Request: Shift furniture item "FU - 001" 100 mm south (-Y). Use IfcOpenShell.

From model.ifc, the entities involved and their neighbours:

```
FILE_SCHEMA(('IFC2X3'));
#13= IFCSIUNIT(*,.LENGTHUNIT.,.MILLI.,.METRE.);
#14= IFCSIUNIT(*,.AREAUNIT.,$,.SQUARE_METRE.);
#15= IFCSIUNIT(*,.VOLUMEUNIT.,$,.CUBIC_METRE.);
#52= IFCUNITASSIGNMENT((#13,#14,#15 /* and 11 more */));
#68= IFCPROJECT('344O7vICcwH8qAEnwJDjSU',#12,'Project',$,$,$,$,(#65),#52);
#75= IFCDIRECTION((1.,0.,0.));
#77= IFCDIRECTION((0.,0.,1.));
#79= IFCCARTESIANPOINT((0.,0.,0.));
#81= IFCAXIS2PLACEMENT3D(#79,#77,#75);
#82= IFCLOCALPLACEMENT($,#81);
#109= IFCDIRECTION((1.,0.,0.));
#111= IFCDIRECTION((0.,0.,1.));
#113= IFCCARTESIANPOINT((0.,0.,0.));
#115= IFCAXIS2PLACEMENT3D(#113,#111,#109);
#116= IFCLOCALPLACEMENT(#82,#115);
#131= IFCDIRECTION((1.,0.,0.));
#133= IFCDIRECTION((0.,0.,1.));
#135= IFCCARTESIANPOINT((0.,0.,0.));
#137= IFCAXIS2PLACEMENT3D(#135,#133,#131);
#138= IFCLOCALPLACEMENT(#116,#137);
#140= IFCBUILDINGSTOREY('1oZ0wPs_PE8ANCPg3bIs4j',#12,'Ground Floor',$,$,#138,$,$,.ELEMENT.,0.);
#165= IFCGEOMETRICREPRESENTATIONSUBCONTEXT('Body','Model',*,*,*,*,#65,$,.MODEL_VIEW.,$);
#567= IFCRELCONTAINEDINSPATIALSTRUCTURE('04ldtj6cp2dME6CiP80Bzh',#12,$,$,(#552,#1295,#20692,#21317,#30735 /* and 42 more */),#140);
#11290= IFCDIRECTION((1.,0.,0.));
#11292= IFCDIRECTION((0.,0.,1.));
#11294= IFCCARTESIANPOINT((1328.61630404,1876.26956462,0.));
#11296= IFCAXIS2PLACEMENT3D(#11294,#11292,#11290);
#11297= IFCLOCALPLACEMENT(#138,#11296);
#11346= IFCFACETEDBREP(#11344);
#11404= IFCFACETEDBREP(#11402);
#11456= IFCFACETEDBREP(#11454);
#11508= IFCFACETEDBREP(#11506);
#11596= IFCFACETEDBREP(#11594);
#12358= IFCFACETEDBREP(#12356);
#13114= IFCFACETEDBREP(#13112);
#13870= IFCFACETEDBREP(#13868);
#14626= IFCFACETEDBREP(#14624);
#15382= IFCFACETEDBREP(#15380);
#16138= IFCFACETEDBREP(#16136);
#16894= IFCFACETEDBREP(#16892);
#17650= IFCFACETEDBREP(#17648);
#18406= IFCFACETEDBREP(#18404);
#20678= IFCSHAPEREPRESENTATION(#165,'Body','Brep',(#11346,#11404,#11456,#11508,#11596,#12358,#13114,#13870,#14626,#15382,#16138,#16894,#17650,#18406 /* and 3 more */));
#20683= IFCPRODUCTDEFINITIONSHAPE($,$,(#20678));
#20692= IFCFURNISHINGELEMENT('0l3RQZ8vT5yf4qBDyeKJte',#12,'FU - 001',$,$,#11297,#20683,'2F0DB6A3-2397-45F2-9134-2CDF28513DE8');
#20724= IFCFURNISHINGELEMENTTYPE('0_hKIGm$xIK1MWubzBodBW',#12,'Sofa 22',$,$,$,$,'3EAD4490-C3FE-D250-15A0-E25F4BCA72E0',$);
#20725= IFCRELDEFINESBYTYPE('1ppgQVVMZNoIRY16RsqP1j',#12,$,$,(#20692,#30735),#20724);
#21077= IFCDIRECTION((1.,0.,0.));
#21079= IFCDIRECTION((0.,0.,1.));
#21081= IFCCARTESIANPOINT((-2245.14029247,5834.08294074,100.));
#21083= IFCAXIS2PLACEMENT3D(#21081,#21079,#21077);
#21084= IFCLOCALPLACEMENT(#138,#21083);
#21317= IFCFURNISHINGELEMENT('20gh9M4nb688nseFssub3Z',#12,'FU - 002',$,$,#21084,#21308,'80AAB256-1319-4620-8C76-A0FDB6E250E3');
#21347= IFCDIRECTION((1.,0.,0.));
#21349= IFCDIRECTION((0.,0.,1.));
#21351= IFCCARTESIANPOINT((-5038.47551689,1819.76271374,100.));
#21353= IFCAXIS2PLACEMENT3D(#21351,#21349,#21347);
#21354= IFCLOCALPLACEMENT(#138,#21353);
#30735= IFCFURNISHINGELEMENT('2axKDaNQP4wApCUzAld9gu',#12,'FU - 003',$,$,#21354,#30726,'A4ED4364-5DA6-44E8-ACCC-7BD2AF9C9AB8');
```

```python
import ifcopenshell
import ifcopenshell.api.geometry
import ifcopenshell.util.placement

model = ifcopenshell.open("model.ifc")

item = model.by_guid("0l3RQZ8vT5yf4qBDyeKJte")
matrix = ifcopenshell.util.placement.get_local_placement(item.ObjectPlacement)
matrix[1, 3] -= 100.0
ifcopenshell.api.geometry.edit_object_placement(model, product=item, matrix=matrix, is_si=False)

print(ifcopenshell.util.placement.get_local_placement(item.ObjectPlacement).round(3) + 0.0)

model.write("model_updated.ifc")
```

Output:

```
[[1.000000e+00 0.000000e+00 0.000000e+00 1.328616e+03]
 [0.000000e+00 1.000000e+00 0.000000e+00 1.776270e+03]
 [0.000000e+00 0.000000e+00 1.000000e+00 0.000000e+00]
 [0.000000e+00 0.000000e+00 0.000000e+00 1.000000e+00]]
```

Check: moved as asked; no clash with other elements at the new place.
